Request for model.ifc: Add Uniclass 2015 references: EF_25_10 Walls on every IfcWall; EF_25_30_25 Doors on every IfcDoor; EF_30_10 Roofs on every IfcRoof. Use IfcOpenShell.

First a look at what the model holds.

```python
import ifcopenshell

model = ifcopenshell.open("model.ifc")
print(model.schema)
print("classifications:", [c.Name for c in model.by_type("IfcClassification")])
for ifc_class in ("IfcDoor", "IfcRoof", "IfcStair", "IfcWall", "IfcWindow"):
    print(ifc_class, len(model.by_type(ifc_class)))
```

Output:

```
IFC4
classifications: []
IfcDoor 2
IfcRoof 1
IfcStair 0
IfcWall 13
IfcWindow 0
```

```python
import ifcopenshell
import ifcopenshell.api.classification

model = ifcopenshell.open("model.ifc")

system = ifcopenshell.api.classification.add_classification(model, classification="Uniclass 2015")

codes = {
    "IfcWall": ("EF_25_10", "Walls"),
    "IfcDoor": ("EF_25_30_25", "Doors"),
    "IfcRoof": ("EF_30_10", "Roofs"),
}
for ifc_class, (code, name) in codes.items():
    products = model.by_type(ifc_class)
    ifcopenshell.api.classification.add_reference(
        model, products=products, classification=system, identification=code, name=name
    )
    print(code, len(products))

model.write("model-out.ifc")
```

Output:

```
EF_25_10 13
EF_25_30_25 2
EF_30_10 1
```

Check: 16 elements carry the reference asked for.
